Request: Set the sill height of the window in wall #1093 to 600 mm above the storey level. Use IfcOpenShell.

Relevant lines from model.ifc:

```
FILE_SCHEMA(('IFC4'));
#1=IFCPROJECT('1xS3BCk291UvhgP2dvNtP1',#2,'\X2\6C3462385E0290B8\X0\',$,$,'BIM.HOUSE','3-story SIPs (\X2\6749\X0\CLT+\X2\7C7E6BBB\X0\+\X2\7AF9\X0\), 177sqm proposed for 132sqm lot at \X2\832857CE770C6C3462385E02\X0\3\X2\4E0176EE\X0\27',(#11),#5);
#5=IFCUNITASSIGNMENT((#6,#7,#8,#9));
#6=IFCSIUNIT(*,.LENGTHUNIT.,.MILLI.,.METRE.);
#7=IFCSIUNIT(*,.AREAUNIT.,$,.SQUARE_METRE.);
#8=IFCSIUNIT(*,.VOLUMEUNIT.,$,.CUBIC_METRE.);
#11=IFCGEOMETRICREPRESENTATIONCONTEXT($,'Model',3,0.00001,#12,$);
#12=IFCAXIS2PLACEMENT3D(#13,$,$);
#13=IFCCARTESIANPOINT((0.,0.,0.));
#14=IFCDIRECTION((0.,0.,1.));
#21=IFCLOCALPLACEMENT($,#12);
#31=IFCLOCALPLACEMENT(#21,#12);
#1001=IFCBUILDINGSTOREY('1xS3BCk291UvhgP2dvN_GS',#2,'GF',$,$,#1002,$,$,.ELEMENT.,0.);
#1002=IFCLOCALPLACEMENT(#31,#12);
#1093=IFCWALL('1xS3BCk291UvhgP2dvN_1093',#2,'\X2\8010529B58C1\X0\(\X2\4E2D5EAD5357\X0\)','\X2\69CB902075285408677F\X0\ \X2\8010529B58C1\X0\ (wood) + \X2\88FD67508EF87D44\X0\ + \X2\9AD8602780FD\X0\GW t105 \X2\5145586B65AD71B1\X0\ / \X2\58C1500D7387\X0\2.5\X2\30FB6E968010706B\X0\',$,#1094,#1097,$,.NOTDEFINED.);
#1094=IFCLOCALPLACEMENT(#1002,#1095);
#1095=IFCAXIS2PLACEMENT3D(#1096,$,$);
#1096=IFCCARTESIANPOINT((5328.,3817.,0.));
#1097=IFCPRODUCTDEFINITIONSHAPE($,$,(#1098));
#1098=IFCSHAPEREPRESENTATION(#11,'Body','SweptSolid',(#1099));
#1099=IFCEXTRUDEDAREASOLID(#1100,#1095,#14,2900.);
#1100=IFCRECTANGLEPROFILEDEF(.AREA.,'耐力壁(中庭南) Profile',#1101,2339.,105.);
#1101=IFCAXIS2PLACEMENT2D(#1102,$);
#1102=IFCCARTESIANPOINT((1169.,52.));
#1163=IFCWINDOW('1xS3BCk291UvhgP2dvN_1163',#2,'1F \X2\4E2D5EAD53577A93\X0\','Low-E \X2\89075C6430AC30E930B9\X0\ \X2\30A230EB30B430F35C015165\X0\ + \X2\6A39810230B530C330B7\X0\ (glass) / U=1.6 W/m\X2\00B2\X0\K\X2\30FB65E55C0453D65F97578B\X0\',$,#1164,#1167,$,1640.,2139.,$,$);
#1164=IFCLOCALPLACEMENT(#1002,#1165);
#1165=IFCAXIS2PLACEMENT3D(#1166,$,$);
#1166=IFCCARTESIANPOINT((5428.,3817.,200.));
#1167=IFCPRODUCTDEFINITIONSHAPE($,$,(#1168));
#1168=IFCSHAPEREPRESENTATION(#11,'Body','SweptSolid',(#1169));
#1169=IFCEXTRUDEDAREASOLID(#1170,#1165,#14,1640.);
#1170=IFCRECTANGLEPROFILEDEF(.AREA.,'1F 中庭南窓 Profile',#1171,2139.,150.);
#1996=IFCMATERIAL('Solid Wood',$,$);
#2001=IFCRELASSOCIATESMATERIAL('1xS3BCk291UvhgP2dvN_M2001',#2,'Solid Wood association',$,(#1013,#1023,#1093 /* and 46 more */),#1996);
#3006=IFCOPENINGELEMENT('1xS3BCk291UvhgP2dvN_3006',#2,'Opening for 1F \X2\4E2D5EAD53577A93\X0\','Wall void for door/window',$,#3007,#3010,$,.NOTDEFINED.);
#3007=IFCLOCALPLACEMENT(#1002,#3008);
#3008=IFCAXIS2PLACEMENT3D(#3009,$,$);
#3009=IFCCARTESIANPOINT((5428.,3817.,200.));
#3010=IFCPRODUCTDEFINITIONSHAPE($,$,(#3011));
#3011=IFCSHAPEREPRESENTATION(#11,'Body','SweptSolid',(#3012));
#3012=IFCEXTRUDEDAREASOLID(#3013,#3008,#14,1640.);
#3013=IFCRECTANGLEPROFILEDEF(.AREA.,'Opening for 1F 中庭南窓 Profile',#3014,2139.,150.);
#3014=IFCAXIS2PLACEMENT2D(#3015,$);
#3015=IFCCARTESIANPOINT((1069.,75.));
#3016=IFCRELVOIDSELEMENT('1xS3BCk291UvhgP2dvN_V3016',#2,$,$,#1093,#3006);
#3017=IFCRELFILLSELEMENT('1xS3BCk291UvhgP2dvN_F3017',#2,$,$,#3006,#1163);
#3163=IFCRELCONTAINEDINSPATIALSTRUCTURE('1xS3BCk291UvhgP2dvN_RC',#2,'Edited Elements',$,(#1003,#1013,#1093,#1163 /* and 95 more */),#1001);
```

```python
import numpy as np
import ifcopenshell
import ifcopenshell.api.geometry
import ifcopenshell.geom
import ifcopenshell.util.element
import ifcopenshell.util.placement
import ifcopenshell.util.shape
import ifcopenshell.util.unit

model = ifcopenshell.open("model.ifc")
unit_scale = ifcopenshell.util.unit.calculate_unit_scale(model)

window = model.by_id(1163)
opening = window.FillsVoids[0].RelatingOpeningElement
storey = ifcopenshell.util.element.get_container(window, ifc_class="IfcBuildingStorey")
level = ifcopenshell.util.placement.get_local_placement(storey.ObjectPlacement)[2, 3]

# The opening's origin need not be at the sill, so measure its lowest point.
shape = ifcopenshell.geom.create_shape(ifcopenshell.geom.settings(), opening)
bottom = ifcopenshell.util.shape.get_shape_bottom_elevation(shape, shape.geometry) / unit_scale
dz = level + 0.6 / unit_scale - bottom

shift = np.array([0.0, 0.0, dz])
# The window is not placed relative to its opening, so move both.
for product in (opening, window):
    matrix = ifcopenshell.util.placement.get_local_placement(product.ObjectPlacement)
    matrix[:3, 3] += shift
    ifcopenshell.api.geometry.edit_object_placement(model, product=product, matrix=matrix, is_si=False)

print(f"moved by {dz * unit_scale:+.3f} m")

model.write("model-out.ifc")
```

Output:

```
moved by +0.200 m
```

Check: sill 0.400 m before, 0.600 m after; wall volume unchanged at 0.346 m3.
